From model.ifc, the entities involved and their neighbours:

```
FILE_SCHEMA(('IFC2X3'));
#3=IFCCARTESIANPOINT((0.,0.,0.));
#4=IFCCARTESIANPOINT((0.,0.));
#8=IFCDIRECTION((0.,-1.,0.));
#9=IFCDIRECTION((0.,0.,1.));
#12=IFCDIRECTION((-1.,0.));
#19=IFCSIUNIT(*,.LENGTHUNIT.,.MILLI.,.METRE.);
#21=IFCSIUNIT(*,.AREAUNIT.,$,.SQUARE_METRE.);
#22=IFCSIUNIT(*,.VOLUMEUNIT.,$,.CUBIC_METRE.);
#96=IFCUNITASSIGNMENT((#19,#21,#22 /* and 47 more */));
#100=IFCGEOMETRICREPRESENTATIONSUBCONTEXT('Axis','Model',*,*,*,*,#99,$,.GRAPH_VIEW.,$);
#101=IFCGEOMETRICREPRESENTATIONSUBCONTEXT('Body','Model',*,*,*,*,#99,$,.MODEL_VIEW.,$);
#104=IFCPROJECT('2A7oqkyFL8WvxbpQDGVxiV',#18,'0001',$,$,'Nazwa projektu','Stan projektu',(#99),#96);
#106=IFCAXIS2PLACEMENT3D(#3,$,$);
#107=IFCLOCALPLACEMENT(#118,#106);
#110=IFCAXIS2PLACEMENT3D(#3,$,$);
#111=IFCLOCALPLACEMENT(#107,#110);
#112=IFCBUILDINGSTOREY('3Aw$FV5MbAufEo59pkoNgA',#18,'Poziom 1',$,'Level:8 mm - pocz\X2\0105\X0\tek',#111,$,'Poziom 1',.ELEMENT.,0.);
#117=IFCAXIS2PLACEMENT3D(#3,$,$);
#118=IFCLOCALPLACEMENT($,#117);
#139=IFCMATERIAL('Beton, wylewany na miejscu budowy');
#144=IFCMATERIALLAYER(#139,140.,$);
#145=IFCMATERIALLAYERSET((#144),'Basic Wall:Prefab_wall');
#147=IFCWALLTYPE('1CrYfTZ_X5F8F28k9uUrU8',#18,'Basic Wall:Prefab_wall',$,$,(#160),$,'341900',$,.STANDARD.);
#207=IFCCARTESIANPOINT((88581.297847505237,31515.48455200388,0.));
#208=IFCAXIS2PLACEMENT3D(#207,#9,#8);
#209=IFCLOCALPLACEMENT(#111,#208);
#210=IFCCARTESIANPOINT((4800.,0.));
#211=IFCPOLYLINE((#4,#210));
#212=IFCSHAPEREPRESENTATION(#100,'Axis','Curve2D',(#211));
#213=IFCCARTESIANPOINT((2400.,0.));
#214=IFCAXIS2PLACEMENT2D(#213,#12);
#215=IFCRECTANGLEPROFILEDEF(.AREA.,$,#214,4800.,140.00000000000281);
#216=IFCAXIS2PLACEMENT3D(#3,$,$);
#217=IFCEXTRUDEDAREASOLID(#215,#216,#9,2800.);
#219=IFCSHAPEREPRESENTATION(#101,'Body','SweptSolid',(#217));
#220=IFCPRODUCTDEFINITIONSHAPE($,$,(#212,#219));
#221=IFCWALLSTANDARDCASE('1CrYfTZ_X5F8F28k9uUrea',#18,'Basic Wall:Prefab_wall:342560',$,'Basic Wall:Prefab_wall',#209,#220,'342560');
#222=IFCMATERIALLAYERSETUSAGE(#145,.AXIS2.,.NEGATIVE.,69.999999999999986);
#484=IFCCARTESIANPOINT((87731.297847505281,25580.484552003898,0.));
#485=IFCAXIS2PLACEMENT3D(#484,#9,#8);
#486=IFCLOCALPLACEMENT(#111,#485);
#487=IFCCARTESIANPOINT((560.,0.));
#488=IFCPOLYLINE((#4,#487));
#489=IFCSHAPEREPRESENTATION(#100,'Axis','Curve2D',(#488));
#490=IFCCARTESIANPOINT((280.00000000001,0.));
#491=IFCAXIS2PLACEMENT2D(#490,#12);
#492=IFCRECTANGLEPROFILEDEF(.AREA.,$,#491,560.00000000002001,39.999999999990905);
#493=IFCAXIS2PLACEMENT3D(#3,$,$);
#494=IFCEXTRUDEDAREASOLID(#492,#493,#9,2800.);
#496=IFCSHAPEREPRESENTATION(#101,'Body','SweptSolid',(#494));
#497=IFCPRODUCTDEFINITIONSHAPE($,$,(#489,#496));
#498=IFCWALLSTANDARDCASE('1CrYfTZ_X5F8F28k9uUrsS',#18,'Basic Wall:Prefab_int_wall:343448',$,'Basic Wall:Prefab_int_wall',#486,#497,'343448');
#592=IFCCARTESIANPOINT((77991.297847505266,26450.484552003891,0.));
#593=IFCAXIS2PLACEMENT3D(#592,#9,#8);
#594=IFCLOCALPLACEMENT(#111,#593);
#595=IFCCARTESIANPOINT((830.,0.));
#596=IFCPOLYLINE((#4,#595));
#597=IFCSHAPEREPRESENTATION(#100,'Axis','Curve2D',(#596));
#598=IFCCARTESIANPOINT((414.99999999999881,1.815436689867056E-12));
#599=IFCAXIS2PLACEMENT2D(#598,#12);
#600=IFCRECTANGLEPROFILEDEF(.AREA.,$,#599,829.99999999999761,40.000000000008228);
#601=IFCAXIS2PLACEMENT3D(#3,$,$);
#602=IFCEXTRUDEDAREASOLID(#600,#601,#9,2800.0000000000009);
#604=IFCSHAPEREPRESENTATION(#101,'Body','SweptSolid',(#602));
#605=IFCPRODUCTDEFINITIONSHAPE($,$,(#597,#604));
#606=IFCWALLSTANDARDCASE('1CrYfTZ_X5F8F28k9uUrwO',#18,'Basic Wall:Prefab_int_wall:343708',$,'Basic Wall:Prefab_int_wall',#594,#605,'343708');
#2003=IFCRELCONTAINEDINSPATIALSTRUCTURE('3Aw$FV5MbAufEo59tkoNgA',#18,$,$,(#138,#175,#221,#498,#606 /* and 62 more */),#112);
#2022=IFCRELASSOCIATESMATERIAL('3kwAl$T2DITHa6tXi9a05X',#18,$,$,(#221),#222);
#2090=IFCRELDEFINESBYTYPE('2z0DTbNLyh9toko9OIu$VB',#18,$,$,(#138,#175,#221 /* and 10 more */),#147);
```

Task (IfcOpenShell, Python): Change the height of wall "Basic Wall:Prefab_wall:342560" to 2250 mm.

```python
import ifcopenshell
import ifcopenshell.geom
import ifcopenshell.util.representation
import ifcopenshell.util.shape
import ifcopenshell.util.unit

model = ifcopenshell.open("model.ifc")
unit_scale = ifcopenshell.util.unit.calculate_unit_scale(model)
settings = ifcopenshell.geom.settings()


def volume(element):
    """Net volume in cubic metres, openings subtracted."""
    shape = ifcopenshell.geom.create_shape(settings, element)
    return ifcopenshell.util.shape.get_volume(shape.geometry)


wall = model.by_guid("1CrYfTZ_X5F8F28k9uUrea")
before = volume(wall)

body = ifcopenshell.util.representation.get_representation(wall, "Model", "Body")
solid = body.Items[0]
old_height = solid.Depth
solid.Depth = 2.25 / unit_scale
after = volume(wall)

print(f"height {old_height:g} -> {solid.Depth:g}, volume {before:.3f} -> {after:.3f} m3")

model.write("model_edited.ifc")
```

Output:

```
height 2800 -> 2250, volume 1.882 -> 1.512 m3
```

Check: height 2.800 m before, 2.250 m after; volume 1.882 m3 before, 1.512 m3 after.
